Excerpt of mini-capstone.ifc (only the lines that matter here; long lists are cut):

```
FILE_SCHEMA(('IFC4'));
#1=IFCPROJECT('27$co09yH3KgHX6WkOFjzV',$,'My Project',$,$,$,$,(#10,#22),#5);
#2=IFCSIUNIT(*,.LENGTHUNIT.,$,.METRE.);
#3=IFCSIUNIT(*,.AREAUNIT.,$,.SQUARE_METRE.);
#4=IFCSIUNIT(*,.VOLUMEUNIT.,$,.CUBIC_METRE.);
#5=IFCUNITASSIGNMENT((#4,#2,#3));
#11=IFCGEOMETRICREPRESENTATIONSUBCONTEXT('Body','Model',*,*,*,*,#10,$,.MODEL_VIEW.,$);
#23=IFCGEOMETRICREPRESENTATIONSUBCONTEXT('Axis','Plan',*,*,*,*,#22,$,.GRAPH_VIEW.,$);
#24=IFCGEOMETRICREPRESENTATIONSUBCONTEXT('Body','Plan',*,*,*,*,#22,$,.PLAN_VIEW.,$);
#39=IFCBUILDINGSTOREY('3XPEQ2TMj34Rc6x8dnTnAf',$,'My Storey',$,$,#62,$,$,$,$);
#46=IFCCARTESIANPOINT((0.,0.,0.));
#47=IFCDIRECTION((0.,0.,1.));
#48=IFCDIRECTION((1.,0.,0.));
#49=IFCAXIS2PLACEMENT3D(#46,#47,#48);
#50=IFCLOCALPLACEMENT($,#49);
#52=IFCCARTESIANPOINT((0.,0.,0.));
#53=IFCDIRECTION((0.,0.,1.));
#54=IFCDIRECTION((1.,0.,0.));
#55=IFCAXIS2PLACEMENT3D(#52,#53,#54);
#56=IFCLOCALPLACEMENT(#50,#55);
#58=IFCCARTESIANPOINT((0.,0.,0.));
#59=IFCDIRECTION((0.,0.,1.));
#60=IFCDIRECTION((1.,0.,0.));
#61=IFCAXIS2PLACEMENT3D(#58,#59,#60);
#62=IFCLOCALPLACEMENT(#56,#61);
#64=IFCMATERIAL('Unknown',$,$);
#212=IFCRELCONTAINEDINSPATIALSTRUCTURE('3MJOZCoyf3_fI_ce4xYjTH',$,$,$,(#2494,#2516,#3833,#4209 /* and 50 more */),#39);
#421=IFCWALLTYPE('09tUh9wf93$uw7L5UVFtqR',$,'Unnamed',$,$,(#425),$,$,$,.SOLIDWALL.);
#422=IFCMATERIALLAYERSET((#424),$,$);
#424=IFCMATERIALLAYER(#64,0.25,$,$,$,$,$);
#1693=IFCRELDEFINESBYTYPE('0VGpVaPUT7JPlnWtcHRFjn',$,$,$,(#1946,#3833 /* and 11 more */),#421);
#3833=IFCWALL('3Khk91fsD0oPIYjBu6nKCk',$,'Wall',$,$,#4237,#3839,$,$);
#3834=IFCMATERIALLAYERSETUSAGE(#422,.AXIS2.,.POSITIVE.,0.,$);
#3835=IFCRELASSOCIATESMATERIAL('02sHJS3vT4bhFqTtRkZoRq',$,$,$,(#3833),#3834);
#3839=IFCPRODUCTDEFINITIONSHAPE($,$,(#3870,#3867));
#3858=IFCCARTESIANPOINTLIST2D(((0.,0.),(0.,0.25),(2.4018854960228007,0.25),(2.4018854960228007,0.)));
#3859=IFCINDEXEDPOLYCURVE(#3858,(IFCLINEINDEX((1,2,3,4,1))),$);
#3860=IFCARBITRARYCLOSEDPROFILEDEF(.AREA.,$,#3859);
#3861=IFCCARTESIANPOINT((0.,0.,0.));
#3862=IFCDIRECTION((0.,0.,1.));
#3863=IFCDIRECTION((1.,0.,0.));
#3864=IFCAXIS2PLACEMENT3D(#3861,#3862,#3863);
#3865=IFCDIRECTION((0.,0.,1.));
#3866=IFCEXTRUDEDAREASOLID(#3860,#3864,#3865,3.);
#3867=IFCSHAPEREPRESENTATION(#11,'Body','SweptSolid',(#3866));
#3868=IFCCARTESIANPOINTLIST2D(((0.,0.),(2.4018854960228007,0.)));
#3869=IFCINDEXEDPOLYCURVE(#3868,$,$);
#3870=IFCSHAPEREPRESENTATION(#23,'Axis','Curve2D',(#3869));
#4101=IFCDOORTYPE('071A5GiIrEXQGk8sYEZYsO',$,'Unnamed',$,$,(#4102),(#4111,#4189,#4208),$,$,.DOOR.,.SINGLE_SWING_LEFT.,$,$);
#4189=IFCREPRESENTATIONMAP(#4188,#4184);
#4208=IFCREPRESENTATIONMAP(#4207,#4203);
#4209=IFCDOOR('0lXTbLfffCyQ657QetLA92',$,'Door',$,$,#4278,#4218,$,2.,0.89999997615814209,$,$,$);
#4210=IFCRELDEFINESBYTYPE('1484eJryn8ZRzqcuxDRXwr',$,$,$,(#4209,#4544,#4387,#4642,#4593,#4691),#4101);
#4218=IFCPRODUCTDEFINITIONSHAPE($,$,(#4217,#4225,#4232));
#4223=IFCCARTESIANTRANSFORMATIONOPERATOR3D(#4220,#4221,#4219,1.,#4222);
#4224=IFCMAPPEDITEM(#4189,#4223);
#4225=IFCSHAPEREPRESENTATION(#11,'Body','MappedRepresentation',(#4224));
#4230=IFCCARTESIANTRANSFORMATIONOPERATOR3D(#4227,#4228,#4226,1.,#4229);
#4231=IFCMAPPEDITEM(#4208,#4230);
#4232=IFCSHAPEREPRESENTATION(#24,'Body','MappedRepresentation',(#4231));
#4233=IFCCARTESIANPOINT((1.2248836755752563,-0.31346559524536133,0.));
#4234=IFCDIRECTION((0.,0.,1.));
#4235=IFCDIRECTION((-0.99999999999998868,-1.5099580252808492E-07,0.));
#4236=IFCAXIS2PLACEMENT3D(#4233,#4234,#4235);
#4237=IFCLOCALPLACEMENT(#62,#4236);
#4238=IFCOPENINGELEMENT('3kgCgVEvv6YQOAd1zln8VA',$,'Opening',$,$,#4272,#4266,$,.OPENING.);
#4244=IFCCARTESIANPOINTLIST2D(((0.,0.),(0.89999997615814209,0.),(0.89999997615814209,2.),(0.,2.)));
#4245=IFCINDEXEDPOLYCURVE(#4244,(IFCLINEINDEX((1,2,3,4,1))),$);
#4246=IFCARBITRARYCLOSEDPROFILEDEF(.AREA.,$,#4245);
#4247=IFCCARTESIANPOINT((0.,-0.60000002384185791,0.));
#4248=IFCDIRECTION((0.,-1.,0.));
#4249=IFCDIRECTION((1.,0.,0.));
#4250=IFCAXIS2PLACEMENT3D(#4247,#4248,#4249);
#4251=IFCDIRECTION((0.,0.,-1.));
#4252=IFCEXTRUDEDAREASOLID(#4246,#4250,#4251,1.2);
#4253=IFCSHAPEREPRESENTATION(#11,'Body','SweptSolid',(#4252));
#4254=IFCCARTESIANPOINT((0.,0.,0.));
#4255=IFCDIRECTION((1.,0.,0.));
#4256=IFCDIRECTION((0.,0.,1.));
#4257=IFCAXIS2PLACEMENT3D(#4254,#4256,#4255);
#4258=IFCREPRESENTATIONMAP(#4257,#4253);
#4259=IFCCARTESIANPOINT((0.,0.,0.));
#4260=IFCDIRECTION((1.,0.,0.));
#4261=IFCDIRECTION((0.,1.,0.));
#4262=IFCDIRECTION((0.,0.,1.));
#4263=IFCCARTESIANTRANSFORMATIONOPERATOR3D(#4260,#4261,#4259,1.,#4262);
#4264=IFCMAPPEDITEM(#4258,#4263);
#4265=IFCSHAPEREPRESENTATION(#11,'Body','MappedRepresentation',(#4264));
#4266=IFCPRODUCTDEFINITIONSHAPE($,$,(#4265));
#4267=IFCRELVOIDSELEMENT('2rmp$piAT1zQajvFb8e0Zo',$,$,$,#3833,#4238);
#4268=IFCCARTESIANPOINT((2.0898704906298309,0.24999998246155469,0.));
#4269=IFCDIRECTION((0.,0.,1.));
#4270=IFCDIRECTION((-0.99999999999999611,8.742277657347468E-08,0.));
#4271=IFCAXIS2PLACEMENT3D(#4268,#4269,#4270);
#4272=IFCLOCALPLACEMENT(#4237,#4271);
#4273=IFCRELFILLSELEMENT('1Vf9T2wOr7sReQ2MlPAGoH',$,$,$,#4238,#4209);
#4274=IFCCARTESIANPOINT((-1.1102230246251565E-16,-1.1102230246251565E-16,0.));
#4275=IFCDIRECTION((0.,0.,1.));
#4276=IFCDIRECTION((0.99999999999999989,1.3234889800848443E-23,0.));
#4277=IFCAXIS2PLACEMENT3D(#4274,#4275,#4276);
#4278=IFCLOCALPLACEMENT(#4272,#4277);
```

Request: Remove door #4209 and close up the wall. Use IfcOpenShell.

```python
import ifcopenshell
import ifcopenshell.api.feature
import ifcopenshell.api.root
import ifcopenshell.geom
import ifcopenshell.util.shape

model = ifcopenshell.open("mini-capstone.ifc")
settings = ifcopenshell.geom.settings()


def volume(element):
    """Net volume in cubic metres, openings subtracted."""
    shape = ifcopenshell.geom.create_shape(settings, element)
    return ifcopenshell.util.shape.get_volume(shape.geometry)


door = model.by_guid("0lXTbLfffCyQ657QetLA92")
opening = door.FillsVoids[0].RelatingOpeningElement
wall = opening.VoidsElements[0].RelatingBuildingElement
before = volume(wall)

ifcopenshell.api.root.remove_product(model, product=door)
ifcopenshell.api.feature.remove_feature(model, feature=opening)

after = volume(wall)

print(f"wall volume {before:.3f} -> {after:.3f} m3")

model.write("mini-capstone_updated.ifc")
```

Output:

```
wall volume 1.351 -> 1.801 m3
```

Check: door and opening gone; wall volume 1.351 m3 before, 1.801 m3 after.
